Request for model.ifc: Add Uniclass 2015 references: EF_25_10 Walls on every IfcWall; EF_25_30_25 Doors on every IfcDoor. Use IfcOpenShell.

First a look at what the model holds.

```python
import ifcopenshell

model = ifcopenshell.open("model.ifc")
print(model.schema)
print("classifications:", [c.Name for c in model.by_type("IfcClassification")])
for ifc_class in ("IfcDoor", "IfcRoof", "IfcStair", "IfcWall", "IfcWindow"):
    print(ifc_class, len(model.by_type(ifc_class)))
```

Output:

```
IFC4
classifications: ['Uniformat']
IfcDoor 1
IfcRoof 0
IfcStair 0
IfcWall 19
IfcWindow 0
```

```python
import ifcopenshell
import ifcopenshell.api.classification

model = ifcopenshell.open("model.ifc")

system = ifcopenshell.api.classification.add_classification(model, classification="Uniclass 2015")

codes = {
    "IfcWall": ("EF_25_10", "Walls"),
    "IfcDoor": ("EF_25_30_25", "Doors"),
}
for ifc_class, (code, name) in codes.items():
    products = model.by_type(ifc_class)
    ifcopenshell.api.classification.add_reference(
        model, products=products, classification=system, identification=code, name=name
    )
    print(code, len(products))

model.write("model_v2.ifc")
```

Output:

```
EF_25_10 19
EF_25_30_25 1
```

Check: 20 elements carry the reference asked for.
